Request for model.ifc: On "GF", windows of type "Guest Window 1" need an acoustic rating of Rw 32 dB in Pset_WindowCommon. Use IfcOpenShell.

First a look at what the model holds.

```python
import ifcopenshell
import ifcopenshell.util.element

model = ifcopenshell.open("model.ifc")
print(model.schema)
storey = next(s for s in model.by_type("IfcBuildingStorey") if s.Name == "GF")
windows = [e for e in ifcopenshell.util.element.get_decomposition(storey) if e.is_a("IfcWindow")]
seen = {}
for e in windows:
    element_type = ifcopenshell.util.element.get_type(e)
    key = (element_type.Name if element_type != e and element_type else None, ifcopenshell.util.element.get_pset(e, "Pset_WindowCommon", "AcousticRating"))
    seen[key] = seen.get(key, 0) + 1
for (name, value), count in sorted(seen.items(), key=str):
    print(count, "x", name, "|", value)
```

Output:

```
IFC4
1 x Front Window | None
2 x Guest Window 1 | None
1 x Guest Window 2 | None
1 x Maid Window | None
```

```python
import ifcopenshell
import ifcopenshell.api.pset
import ifcopenshell.util.element

model = ifcopenshell.open("model.ifc")

storey = next(s for s in model.by_type("IfcBuildingStorey") if s.Name == "GF")
windows = [e for e in ifcopenshell.util.element.get_decomposition(storey) if e.is_a("IfcWindow")]

count = 0
for e in windows:
    element_type = ifcopenshell.util.element.get_type(e)
    if element_type in (None, e) or element_type.Name != "Guest Window 1":
        continue
    # add_pset returns the element's existing set when there is one.
    pset = ifcopenshell.api.pset.add_pset(model, product=e, name="Pset_WindowCommon")
    ifcopenshell.api.pset.edit_pset(model, pset=pset, properties={"AcousticRating": "Rw 32 dB"})
    count += 1

print(count, "windows updated")

model.write("model_rev.ifc")
```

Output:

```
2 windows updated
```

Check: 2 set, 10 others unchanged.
